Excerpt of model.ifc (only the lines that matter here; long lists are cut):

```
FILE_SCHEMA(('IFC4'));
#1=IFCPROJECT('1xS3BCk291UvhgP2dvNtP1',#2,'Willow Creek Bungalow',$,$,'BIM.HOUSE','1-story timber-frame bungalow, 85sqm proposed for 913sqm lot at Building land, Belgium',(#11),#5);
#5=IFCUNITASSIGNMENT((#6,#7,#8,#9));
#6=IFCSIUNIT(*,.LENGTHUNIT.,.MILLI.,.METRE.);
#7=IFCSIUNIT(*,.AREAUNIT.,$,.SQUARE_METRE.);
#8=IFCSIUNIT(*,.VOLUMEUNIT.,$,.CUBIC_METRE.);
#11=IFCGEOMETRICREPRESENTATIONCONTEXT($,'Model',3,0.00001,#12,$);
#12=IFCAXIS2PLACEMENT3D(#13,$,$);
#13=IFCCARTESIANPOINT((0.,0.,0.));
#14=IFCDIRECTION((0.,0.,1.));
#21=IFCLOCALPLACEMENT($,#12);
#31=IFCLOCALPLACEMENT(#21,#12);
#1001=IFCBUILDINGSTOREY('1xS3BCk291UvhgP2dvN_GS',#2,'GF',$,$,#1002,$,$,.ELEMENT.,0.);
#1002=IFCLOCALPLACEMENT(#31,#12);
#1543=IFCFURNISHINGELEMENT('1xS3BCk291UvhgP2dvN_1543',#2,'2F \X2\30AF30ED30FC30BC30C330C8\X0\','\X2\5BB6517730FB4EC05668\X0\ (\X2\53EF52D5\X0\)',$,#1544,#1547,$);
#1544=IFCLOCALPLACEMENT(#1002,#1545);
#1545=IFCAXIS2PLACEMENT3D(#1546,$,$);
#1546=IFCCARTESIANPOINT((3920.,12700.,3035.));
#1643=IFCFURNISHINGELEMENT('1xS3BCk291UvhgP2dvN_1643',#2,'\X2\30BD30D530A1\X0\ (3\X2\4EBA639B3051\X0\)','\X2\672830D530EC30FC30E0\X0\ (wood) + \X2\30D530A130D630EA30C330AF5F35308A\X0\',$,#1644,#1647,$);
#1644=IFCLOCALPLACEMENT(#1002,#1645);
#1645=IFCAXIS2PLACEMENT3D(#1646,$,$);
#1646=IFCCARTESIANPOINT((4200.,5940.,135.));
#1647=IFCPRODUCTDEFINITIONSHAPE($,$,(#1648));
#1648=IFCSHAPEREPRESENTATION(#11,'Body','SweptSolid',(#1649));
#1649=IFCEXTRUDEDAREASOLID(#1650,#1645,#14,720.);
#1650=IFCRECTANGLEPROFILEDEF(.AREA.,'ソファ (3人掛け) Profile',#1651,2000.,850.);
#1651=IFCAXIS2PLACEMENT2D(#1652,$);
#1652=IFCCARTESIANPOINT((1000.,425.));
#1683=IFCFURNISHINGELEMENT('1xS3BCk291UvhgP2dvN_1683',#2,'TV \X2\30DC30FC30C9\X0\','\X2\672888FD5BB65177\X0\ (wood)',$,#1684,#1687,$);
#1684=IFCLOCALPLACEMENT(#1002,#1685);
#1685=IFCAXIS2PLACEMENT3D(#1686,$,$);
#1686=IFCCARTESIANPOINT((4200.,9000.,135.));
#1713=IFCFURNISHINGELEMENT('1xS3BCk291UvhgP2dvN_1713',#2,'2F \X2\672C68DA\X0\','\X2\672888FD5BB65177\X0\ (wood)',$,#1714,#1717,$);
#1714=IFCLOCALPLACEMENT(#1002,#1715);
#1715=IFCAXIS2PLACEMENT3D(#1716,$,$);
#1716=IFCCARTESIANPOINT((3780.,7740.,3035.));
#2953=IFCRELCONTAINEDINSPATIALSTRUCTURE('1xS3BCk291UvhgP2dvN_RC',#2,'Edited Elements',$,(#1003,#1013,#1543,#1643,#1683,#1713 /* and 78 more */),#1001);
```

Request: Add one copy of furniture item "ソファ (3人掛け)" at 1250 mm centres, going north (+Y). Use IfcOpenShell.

```python
import numpy as np
import ifcopenshell
import ifcopenshell.api.geometry
import ifcopenshell.api.root
import ifcopenshell.util.element
import ifcopenshell.util.placement
import ifcopenshell.util.unit

model = ifcopenshell.open("model.ifc")
unit_scale = ifcopenshell.util.unit.calculate_unit_scale(model)


def reuse_history(source, copy):
    """copy_class also copies each property set's owner history, people and application; keep the originals."""
    for rel in copy.IsDefinedBy:
        if rel.is_a("IfcRelDefinesByProperties") and (history := rel.RelatingPropertyDefinition.OwnerHistory):
            rel.RelatingPropertyDefinition.OwnerHistory = source.OwnerHistory
            ifcopenshell.util.element.remove_deep2(model, history)


source = model.by_guid("1xS3BCk291UvhgP2dvN_1643")
base = ifcopenshell.util.placement.get_local_placement(source.ObjectPlacement)
step = np.array([0.0, 1.0, 0.0]) * 1.25 / unit_scale

for i in range(1, 2):
    copy = ifcopenshell.api.root.copy_class(model, product=source)
    copy.Representation = ifcopenshell.util.element.copy_deep(
        model, source.Representation, exclude=["IfcGeometricRepresentationContext", "IfcRepresentationMap"]
    )
    reuse_history(source, copy)
    matrix = base.copy()
    matrix[:3, 3] += i * step
    print("added at", matrix[:3, 3].round(3) + 0.0)
    ifcopenshell.api.geometry.edit_object_placement(model, product=copy, matrix=matrix, is_si=False)

model.write("model_updated.ifc")
```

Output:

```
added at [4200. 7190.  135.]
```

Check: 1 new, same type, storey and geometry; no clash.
